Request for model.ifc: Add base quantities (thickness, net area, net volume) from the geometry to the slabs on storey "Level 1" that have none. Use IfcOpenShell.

First a look at what the model holds.

```python
import ifcopenshell
import ifcopenshell.util.element
import ifcopenshell.util.unit

model = ifcopenshell.open("model.ifc")
print(model.schema)
for unit_type in ("LENGTHUNIT", "AREAUNIT", "VOLUMEUNIT"):
    print(unit_type, ifcopenshell.util.unit.calculate_unit_scale(model, unit_type))
storey = next(s for s in model.by_type("IfcBuildingStorey") if s.Name == "Level 1")
slabs = [e for e in ifcopenshell.util.element.get_decomposition(storey) if e.is_a("IfcSlab")]
for e in sorted(slabs, key=lambda e: e.id()):
    print(e.id(), e.is_a(), e.Name, list(ifcopenshell.util.element.get_psets(e, qtos_only=True)), sep=" | ")
```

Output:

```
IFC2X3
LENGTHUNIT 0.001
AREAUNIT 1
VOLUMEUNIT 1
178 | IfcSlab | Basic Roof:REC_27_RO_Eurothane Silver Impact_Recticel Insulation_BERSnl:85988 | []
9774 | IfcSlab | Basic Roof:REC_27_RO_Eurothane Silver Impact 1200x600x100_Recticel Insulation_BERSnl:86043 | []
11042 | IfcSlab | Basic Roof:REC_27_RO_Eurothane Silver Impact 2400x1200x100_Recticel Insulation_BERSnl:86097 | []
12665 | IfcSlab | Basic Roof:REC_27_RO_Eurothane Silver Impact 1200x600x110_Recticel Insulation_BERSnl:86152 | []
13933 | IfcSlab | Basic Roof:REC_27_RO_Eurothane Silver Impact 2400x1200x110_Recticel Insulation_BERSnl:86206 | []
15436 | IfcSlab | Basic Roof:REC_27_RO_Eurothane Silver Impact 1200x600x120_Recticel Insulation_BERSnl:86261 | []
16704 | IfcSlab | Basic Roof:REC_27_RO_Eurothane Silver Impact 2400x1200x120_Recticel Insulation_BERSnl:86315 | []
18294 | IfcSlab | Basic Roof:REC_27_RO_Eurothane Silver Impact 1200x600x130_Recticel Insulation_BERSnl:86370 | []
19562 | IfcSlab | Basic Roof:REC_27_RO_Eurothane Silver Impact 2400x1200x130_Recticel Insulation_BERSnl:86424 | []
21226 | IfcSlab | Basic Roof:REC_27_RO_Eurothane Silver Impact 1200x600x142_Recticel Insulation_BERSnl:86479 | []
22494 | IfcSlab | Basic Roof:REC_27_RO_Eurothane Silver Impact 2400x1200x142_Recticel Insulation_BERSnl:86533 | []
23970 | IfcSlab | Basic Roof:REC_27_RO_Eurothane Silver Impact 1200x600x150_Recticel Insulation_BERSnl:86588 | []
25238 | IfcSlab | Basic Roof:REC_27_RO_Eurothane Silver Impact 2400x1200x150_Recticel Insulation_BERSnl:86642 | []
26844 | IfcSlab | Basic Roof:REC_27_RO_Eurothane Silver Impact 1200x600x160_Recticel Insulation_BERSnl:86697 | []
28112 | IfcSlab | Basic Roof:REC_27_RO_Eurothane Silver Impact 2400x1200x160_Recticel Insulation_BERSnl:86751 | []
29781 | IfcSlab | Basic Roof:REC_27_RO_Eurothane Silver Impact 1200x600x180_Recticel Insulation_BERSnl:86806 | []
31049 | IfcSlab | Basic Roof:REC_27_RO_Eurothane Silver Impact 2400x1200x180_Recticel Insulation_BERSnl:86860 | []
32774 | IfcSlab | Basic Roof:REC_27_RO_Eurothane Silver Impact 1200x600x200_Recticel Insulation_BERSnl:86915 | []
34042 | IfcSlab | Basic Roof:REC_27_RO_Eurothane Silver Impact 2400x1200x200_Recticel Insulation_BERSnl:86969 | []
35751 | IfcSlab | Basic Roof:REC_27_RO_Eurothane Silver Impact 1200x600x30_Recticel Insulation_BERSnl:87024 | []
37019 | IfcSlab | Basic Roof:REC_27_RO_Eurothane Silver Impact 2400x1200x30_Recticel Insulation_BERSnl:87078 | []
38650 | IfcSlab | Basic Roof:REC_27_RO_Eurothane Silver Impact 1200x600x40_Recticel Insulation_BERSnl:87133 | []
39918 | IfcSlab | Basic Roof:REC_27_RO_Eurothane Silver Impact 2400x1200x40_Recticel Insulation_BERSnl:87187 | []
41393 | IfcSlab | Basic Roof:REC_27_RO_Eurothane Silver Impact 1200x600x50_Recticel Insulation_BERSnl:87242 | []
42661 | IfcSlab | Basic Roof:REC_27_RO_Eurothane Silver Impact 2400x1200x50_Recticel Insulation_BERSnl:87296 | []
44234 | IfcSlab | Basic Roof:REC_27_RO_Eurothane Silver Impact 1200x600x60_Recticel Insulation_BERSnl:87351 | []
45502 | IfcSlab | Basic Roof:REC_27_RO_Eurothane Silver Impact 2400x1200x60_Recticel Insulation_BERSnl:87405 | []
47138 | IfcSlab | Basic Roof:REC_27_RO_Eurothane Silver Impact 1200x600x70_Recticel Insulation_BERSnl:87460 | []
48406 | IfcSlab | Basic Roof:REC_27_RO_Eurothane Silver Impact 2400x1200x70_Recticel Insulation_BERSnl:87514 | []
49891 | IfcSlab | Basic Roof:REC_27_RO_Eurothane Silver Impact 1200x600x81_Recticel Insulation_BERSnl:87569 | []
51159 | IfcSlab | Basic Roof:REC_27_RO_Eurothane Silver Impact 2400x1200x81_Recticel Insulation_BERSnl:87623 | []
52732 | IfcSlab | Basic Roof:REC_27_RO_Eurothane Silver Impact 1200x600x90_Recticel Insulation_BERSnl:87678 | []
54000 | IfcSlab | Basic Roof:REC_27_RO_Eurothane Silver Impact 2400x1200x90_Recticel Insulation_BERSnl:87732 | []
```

```python
import ifcopenshell
import ifcopenshell.api.pset
import ifcopenshell.geom
import ifcopenshell.util.element
import ifcopenshell.util.shape
import ifcopenshell.util.unit

model = ifcopenshell.open("model.ifc")
unit_scale = ifcopenshell.util.unit.calculate_unit_scale(model)
area_scale = ifcopenshell.util.unit.calculate_unit_scale(model, "AREAUNIT")
volume_scale = ifcopenshell.util.unit.calculate_unit_scale(model, "VOLUMEUNIT")
settings = ifcopenshell.geom.settings()

storey = next(s for s in model.by_type("IfcBuildingStorey") if s.Name == "Level 1")
slabs = [e for e in ifcopenshell.util.element.get_decomposition(storey) if e.is_a("IfcSlab")]

for e in sorted(slabs, key=lambda e: e.id()):
    if ifcopenshell.util.element.get_psets(e, qtos_only=True, should_inherit=False):
        continue
    # Geometry comes back in metres, in the element's own axes.
    shape = ifcopenshell.geom.create_shape(settings, e)
    values = {
        "Width": ifcopenshell.util.shape.get_z(shape.geometry) / unit_scale,
        "NetArea": ifcopenshell.util.shape.get_footprint_area(shape.geometry) / area_scale,
        "NetVolume": ifcopenshell.util.shape.get_volume(shape.geometry) / volume_scale,
    }
    qto = ifcopenshell.api.pset.add_qto(model, product=e, name="BaseQuantities")
    ifcopenshell.api.pset.edit_qto(model, qto=qto, properties=values)
    print(e.id(), {k: round(v, 3) for k, v in values.items()})

model.write("model_rev.ifc")
```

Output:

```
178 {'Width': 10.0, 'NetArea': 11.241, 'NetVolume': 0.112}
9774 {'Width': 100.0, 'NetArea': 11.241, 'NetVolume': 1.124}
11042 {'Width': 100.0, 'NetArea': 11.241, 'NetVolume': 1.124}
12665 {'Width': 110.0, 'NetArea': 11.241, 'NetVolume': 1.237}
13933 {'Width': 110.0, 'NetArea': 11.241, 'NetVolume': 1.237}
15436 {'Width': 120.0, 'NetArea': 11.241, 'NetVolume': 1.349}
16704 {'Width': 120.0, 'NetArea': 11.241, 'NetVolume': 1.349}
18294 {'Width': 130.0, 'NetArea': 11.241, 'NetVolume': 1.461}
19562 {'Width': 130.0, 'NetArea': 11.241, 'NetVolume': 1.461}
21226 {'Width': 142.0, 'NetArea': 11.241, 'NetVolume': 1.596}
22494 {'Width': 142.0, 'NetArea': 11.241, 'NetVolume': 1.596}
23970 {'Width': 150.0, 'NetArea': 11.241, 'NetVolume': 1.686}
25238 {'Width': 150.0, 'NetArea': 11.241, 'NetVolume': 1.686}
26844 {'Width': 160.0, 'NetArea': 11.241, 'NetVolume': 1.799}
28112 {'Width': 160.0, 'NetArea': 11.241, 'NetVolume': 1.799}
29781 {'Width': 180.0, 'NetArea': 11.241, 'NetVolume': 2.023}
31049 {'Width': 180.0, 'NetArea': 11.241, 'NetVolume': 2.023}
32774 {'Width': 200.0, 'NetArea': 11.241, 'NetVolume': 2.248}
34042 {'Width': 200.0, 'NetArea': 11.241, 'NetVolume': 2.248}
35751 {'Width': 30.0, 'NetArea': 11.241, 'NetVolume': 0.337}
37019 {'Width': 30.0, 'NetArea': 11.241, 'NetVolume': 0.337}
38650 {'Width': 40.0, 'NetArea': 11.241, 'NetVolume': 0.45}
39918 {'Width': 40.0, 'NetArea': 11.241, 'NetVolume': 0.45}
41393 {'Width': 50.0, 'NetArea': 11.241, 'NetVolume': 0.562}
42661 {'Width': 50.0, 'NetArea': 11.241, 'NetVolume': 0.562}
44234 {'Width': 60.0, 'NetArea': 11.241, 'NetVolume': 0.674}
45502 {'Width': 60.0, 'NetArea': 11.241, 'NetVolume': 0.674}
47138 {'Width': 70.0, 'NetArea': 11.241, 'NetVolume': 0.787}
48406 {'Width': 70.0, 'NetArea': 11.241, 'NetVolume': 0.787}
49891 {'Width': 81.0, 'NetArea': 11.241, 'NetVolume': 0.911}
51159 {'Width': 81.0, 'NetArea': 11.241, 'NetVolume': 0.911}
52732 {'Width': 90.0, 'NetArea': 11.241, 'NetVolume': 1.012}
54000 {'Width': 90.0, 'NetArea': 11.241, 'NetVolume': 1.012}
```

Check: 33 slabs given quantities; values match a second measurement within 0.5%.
